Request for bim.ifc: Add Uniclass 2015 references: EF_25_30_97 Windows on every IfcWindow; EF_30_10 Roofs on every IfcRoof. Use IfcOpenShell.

First a look at what the model holds.

```python
import ifcopenshell

model = ifcopenshell.open("bim.ifc")
print(model.schema)
print("classifications:", [c.Name for c in model.by_type("IfcClassification")])
for ifc_class in ("IfcDoor", "IfcRoof", "IfcStair", "IfcWall", "IfcWindow"):
    print(ifc_class, len(model.by_type(ifc_class)))
```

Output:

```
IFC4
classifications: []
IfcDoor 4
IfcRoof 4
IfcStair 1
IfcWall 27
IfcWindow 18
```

```python
import ifcopenshell
import ifcopenshell.api.classification

model = ifcopenshell.open("bim.ifc")

system = ifcopenshell.api.classification.add_classification(model, classification="Uniclass 2015")

codes = {
    "IfcWindow": ("EF_25_30_97", "Windows"),
    "IfcRoof": ("EF_30_10", "Roofs"),
}
for ifc_class, (code, name) in codes.items():
    products = model.by_type(ifc_class)
    ifcopenshell.api.classification.add_reference(
        model, products=products, classification=system, identification=code, name=name
    )
    print(code, len(products))

model.write("bim_updated.ifc")
```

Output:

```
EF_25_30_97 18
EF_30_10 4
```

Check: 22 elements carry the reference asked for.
